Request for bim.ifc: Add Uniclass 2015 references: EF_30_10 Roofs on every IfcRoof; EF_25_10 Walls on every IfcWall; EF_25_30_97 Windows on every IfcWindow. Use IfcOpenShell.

First a look at what the model holds.

```python
import ifcopenshell

model = ifcopenshell.open("bim.ifc")
print(model.schema)
print("classifications:", [c.Name for c in model.by_type("IfcClassification")])
for ifc_class in ("IfcDoor", "IfcRoof", "IfcStair", "IfcWall", "IfcWindow"):
    print(ifc_class, len(model.by_type(ifc_class)))
```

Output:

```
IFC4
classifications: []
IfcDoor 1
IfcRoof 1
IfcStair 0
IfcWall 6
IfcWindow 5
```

```python
import ifcopenshell
import ifcopenshell.api.classification

model = ifcopenshell.open("bim.ifc")

system = ifcopenshell.api.classification.add_classification(model, classification="Uniclass 2015")

codes = {
    "IfcRoof": ("EF_30_10", "Roofs"),
    "IfcWall": ("EF_25_10", "Walls"),
    "IfcWindow": ("EF_25_30_97", "Windows"),
}
for ifc_class, (code, name) in codes.items():
    products = model.by_type(ifc_class)
    ifcopenshell.api.classification.add_reference(
        model, products=products, classification=system, identification=code, name=name
    )
    print(code, len(products))

model.write("bim_edited.ifc")
```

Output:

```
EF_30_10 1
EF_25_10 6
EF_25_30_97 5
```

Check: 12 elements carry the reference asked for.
